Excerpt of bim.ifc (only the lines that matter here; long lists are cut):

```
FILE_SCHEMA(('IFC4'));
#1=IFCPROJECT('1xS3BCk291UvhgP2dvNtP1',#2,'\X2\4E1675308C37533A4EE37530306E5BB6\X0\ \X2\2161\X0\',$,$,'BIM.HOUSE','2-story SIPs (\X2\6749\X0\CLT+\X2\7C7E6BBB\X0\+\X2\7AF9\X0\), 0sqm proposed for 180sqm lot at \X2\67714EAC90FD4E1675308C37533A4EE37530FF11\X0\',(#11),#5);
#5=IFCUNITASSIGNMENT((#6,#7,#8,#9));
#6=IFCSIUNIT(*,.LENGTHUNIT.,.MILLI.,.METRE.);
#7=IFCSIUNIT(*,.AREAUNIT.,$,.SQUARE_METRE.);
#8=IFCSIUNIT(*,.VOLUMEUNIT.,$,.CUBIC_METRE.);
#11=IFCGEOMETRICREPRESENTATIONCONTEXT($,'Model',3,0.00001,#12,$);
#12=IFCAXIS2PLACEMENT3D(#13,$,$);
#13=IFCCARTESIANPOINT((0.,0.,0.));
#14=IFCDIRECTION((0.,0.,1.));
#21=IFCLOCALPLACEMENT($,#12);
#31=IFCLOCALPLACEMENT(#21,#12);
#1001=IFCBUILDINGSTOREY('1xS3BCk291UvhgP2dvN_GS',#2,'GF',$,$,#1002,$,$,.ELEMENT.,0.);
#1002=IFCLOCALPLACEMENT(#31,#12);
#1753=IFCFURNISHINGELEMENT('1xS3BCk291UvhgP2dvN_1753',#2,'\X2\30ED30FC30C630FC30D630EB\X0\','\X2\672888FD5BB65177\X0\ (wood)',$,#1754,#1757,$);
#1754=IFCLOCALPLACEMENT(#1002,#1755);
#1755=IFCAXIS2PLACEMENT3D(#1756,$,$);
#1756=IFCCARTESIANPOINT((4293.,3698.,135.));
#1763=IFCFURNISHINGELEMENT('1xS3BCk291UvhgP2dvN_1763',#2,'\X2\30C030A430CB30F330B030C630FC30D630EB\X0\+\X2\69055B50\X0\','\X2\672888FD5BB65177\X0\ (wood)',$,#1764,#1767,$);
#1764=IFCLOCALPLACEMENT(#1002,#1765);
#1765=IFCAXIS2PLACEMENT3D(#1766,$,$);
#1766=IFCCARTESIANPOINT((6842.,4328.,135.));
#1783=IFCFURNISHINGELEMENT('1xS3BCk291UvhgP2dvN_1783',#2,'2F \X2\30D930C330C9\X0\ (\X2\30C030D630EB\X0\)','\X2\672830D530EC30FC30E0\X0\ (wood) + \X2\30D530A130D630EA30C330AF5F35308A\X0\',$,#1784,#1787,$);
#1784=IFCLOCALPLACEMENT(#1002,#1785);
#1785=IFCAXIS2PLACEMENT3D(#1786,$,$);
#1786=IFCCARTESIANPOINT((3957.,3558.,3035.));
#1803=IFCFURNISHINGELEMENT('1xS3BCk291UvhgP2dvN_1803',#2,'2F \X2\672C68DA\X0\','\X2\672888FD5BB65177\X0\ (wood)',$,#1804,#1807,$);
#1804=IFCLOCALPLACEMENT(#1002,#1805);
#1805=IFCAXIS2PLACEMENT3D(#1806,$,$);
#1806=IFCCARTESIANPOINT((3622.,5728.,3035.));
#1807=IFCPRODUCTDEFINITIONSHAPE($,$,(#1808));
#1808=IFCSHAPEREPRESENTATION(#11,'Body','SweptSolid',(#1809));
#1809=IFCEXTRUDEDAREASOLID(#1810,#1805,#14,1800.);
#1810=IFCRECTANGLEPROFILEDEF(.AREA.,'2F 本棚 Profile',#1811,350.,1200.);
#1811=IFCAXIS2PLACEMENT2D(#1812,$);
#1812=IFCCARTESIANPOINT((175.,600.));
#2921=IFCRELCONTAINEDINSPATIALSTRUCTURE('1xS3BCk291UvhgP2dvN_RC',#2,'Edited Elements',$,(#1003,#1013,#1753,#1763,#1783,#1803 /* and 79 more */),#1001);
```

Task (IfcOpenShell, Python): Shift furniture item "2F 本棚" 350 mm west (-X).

```python
import ifcopenshell
import ifcopenshell.api.geometry
import ifcopenshell.util.placement

model = ifcopenshell.open("bim.ifc")

item = model.by_guid("1xS3BCk291UvhgP2dvN_1803")
matrix = ifcopenshell.util.placement.get_local_placement(item.ObjectPlacement)
matrix[0, 3] -= 350.0
ifcopenshell.api.geometry.edit_object_placement(model, product=item, matrix=matrix, is_si=False)

print(ifcopenshell.util.placement.get_local_placement(item.ObjectPlacement).round(3) + 0.0)

model.write("bim_rev.ifc")
```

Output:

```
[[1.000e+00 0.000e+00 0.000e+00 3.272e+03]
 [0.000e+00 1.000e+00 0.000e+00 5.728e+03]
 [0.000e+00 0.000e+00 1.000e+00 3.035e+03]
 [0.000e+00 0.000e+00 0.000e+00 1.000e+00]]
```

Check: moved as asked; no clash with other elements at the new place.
